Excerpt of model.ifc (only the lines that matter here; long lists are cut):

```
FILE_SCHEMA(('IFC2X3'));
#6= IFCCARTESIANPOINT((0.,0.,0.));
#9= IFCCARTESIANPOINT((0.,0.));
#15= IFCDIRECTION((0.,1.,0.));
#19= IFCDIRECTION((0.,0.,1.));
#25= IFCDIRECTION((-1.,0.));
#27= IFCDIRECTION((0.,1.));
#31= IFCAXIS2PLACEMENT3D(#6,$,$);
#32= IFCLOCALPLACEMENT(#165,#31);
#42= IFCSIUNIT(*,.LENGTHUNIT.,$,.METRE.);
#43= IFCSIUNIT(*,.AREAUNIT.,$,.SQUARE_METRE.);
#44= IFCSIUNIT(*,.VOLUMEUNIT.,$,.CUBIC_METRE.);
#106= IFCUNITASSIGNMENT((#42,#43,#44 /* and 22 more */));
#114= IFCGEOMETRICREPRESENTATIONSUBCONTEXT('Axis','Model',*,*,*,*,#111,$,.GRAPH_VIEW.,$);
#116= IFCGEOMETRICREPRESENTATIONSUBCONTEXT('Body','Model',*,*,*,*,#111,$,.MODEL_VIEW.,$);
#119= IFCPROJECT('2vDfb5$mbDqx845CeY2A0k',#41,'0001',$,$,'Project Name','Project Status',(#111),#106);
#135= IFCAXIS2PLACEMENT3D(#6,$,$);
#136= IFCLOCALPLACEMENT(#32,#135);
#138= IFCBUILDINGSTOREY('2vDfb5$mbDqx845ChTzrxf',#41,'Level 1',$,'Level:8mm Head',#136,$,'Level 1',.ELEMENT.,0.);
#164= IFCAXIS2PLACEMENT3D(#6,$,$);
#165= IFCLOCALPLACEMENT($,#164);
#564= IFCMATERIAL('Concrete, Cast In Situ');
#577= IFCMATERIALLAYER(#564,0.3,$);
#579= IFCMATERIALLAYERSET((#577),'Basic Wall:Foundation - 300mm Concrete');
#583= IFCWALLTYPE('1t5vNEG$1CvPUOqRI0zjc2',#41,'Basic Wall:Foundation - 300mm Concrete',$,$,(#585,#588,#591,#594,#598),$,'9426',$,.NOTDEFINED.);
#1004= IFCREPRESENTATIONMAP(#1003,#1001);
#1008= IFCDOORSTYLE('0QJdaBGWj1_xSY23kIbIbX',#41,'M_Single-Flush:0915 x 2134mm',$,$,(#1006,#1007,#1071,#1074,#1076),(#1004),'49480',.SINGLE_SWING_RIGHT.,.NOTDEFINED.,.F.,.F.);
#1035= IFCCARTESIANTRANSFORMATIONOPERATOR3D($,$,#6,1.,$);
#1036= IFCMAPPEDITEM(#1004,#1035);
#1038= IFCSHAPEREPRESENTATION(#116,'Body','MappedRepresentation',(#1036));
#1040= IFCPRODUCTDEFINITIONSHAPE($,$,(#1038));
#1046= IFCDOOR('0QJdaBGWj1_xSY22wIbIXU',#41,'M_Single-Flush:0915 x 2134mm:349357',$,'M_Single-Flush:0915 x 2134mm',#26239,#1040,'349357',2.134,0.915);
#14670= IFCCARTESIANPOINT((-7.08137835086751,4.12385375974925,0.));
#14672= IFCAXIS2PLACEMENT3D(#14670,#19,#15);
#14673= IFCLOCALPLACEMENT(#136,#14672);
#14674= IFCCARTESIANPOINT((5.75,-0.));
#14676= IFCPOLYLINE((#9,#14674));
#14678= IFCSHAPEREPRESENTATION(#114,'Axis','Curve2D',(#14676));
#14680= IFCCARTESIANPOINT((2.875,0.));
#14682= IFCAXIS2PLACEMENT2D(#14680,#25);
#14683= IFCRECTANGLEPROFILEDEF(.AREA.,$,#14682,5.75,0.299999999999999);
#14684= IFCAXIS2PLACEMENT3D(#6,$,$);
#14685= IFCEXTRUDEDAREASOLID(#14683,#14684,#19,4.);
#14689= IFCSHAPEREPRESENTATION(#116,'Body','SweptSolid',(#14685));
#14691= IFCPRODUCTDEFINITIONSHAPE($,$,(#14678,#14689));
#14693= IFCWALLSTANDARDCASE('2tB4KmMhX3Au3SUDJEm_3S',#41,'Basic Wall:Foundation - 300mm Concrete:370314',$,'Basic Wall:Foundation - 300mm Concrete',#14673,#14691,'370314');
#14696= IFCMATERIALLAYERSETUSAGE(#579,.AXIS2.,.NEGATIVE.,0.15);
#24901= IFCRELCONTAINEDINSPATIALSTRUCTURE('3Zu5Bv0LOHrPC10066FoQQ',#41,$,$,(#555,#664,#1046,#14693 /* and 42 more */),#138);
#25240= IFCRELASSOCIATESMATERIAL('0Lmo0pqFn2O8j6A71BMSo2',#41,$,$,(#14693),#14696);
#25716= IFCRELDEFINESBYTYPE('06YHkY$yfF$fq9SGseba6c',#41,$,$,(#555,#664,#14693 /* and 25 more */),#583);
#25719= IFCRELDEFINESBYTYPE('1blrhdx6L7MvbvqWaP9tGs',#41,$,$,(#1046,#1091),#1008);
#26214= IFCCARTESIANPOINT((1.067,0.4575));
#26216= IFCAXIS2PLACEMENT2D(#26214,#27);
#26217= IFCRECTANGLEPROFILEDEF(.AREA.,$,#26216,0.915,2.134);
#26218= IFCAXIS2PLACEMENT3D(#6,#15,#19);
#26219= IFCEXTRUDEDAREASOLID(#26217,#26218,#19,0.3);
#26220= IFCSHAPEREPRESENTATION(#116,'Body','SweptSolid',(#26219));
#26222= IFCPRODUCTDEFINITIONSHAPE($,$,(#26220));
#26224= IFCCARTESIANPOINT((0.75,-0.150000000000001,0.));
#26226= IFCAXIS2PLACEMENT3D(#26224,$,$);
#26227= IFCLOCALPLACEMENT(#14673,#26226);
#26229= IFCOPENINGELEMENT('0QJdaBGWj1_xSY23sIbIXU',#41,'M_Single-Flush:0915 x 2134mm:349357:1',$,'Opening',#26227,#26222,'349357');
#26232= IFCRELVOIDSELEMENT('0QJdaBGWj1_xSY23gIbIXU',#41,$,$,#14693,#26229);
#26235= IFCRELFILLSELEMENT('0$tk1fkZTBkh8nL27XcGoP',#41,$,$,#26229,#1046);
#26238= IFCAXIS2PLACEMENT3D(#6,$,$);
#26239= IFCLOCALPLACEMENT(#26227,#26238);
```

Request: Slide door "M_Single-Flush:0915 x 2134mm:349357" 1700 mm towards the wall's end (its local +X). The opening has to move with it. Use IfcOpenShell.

```python
import ifcopenshell
import ifcopenshell.api.geometry
import ifcopenshell.util.placement

model = ifcopenshell.open("model.ifc")

door = model.by_id(1046)
opening = door.FillsVoids[0].RelatingOpeningElement
wall = opening.VoidsElements[0].RelatingBuildingElement

wall_matrix = ifcopenshell.util.placement.get_local_placement(wall.ObjectPlacement)
shift = wall_matrix[:3, 0] * 1.7
before = ifcopenshell.util.placement.get_local_placement(door.ObjectPlacement)[:3, 3].copy()

# The door is placed relative to its opening, so it follows when the opening moves.
matrix = ifcopenshell.util.placement.get_local_placement(opening.ObjectPlacement)
matrix[:3, 3] += shift
ifcopenshell.api.geometry.edit_object_placement(
    model, product=opening, matrix=matrix, is_si=False, should_transform_children=True
)

after = ifcopenshell.util.placement.get_local_placement(door.ObjectPlacement)[:3, 3]
print("door moved by", (after - before).round(3) + 0.0)

model.write("model-out.ifc")
```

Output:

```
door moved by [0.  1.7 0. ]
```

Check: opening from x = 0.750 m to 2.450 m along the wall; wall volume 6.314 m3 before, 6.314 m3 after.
